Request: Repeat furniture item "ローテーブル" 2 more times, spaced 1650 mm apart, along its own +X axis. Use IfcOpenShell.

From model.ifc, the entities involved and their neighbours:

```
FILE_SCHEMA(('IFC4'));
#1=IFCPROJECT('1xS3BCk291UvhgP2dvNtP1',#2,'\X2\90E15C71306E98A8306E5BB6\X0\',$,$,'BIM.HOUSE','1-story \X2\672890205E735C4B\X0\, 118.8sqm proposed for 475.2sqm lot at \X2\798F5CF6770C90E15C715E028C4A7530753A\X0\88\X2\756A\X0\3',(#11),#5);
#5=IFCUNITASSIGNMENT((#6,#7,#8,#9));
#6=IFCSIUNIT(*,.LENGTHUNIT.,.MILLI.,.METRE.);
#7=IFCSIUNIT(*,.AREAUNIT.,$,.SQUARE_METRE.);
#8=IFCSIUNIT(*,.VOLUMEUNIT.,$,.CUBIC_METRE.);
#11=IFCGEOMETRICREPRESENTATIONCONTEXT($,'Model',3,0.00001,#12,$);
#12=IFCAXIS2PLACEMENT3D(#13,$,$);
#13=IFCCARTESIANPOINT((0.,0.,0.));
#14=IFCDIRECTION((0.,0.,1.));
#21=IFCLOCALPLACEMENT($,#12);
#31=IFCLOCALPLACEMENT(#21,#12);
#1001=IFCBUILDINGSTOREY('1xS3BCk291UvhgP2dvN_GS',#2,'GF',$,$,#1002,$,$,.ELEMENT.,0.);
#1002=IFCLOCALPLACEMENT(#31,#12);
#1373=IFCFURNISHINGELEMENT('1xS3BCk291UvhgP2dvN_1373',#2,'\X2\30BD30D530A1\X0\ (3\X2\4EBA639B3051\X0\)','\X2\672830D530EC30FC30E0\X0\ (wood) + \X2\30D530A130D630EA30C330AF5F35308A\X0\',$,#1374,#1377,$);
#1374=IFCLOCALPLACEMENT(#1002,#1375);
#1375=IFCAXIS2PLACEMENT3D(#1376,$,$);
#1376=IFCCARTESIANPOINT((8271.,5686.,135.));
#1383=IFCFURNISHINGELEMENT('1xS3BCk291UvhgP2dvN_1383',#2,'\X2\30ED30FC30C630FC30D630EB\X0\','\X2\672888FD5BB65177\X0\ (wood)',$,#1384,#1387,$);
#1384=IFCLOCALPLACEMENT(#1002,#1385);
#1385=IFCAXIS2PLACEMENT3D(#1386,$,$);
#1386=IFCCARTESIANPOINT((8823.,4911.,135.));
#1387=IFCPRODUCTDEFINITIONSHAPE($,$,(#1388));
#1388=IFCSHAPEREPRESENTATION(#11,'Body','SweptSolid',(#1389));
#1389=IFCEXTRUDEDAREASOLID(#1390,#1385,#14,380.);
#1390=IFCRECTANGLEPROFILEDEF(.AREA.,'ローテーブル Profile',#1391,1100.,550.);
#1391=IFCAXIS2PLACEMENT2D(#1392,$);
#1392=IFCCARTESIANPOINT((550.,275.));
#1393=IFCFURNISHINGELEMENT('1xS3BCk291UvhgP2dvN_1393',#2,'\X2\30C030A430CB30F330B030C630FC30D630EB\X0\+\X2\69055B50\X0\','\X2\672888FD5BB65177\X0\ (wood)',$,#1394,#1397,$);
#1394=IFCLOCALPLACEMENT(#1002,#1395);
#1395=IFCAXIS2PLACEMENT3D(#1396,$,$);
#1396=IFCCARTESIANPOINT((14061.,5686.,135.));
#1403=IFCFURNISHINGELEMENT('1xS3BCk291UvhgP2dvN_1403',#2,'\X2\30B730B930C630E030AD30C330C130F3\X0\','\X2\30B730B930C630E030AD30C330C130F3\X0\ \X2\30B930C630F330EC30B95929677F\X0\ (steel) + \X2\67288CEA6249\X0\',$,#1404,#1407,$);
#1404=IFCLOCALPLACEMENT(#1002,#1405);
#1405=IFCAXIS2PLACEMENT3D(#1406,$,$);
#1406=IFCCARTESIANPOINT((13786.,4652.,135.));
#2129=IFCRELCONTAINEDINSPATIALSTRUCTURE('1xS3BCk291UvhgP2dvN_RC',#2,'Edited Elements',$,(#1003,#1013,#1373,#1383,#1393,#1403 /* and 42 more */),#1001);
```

```python
import ifcopenshell
import ifcopenshell.api.geometry
import ifcopenshell.api.root
import ifcopenshell.util.element
import ifcopenshell.util.placement

model = ifcopenshell.open("model.ifc")


def reuse_history(source, copy):
    """copy_class also copies each property set's owner history, people and application; keep the originals."""
    for rel in copy.IsDefinedBy:
        if rel.is_a("IfcRelDefinesByProperties") and (history := rel.RelatingPropertyDefinition.OwnerHistory):
            rel.RelatingPropertyDefinition.OwnerHistory = source.OwnerHistory
            ifcopenshell.util.element.remove_deep2(model, history)


source = model.by_guid("1xS3BCk291UvhgP2dvN_1383")
base = ifcopenshell.util.placement.get_local_placement(source.ObjectPlacement)
step = base[:3, 0] * 1650.0

for i in range(1, 3):
    copy = ifcopenshell.api.root.copy_class(model, product=source)
    copy.Representation = ifcopenshell.util.element.copy_deep(
        model, source.Representation, exclude=["IfcGeometricRepresentationContext", "IfcRepresentationMap"]
    )
    reuse_history(source, copy)
    matrix = base.copy()
    matrix[:3, 3] += i * step
    print("added at", matrix[:3, 3].round(3) + 0.0)
    ifcopenshell.api.geometry.edit_object_placement(model, product=copy, matrix=matrix, is_si=False)

model.write("model_v2.ifc")
```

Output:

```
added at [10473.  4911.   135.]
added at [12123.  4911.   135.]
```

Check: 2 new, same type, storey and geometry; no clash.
